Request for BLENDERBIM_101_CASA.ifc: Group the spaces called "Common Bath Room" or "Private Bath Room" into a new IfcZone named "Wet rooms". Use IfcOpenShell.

First a look at what the model holds.

```python
import ifcopenshell

model = ifcopenshell.open("BLENDERBIM_101_CASA.ifc")
print(model.schema)
seen = {}
for space in model.by_type("IfcSpace"):
    seen[space.Name] = seen.get(space.Name, 0) + 1
for name, count in sorted(seen.items(), key=str):
    print(count, "x", name)
print("zones:", [z.Name for z in model.by_type("IfcZone")][:20])
```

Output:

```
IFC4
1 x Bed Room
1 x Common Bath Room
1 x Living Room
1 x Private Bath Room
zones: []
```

```python
import ifcopenshell
import ifcopenshell.api.group
import ifcopenshell.api.root

model = ifcopenshell.open("BLENDERBIM_101_CASA.ifc")

names = {"Common Bath Room", "Private Bath Room"}
spaces = [s for s in model.by_type("IfcSpace") if s.Name in names]

zone = ifcopenshell.api.root.create_entity(model, ifc_class="IfcZone", name="Wet rooms")
ifcopenshell.api.group.assign_group(model, products=spaces, group=zone)
print(len(spaces), "spaces in", zone.Name)

model.write("BLENDERBIM_101_CASA-out.ifc")
```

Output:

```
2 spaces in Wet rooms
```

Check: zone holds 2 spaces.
